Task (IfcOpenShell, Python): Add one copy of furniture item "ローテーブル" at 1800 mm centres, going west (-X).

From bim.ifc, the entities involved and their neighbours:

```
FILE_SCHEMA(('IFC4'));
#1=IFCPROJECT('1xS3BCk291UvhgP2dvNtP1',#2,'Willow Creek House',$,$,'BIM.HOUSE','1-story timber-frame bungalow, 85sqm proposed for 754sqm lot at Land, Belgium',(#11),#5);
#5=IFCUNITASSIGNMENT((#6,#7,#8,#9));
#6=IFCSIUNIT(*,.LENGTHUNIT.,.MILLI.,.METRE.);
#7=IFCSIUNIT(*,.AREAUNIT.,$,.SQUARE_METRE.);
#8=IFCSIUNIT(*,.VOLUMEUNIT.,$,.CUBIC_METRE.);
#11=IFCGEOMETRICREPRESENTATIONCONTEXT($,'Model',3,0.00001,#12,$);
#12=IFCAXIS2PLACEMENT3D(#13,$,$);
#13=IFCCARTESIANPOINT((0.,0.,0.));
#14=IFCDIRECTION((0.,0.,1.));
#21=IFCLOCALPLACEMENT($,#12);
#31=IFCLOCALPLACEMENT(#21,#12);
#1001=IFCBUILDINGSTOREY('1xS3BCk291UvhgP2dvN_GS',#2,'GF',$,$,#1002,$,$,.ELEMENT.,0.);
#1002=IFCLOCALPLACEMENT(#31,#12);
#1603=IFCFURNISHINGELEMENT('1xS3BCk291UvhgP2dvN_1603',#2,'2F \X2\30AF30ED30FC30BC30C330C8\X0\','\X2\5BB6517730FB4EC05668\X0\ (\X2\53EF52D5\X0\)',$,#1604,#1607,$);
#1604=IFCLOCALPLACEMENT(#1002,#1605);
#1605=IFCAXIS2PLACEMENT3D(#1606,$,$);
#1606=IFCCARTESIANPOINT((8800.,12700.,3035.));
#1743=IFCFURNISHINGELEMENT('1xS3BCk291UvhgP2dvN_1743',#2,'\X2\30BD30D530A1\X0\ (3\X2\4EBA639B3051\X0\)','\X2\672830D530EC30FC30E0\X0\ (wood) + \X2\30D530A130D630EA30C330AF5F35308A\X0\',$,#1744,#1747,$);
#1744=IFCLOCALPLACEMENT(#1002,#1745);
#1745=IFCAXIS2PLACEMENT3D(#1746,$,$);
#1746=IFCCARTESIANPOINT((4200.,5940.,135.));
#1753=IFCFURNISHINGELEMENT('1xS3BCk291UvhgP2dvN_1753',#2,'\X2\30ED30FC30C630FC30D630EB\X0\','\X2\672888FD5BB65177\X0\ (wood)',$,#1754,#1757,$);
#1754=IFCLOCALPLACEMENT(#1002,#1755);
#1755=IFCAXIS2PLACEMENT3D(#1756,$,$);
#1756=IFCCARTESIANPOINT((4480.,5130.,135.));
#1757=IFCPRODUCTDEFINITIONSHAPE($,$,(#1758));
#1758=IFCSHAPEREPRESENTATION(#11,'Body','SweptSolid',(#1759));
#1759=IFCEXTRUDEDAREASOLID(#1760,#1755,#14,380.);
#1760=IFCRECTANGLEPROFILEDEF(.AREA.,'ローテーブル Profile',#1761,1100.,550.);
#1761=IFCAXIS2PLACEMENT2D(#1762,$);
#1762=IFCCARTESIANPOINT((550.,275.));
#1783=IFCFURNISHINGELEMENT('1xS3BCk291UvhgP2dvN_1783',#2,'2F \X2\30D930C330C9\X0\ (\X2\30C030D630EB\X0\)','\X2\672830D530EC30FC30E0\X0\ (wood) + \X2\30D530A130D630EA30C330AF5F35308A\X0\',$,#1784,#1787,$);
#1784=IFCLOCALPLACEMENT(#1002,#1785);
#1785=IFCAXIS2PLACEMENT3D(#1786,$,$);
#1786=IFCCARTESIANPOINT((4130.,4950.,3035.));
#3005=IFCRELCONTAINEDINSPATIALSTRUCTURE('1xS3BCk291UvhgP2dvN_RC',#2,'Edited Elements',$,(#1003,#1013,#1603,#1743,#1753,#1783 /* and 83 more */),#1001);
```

```python
import numpy as np
import ifcopenshell
import ifcopenshell.api.geometry
import ifcopenshell.api.root
import ifcopenshell.util.element
import ifcopenshell.util.placement
import ifcopenshell.util.unit

model = ifcopenshell.open("bim.ifc")
unit_scale = ifcopenshell.util.unit.calculate_unit_scale(model)


def reuse_history(source, copy):
    """copy_class also copies each property set's owner history, people and application; keep the originals."""
    for rel in copy.IsDefinedBy:
        if rel.is_a("IfcRelDefinesByProperties") and (history := rel.RelatingPropertyDefinition.OwnerHistory):
            rel.RelatingPropertyDefinition.OwnerHistory = source.OwnerHistory
            ifcopenshell.util.element.remove_deep2(model, history)


source = model.by_guid("1xS3BCk291UvhgP2dvN_1753")
base = ifcopenshell.util.placement.get_local_placement(source.ObjectPlacement)
step = np.array([-1.0, 0.0, 0.0]) * 1.8 / unit_scale

for i in range(1, 2):
    copy = ifcopenshell.api.root.copy_class(model, product=source)
    copy.Representation = ifcopenshell.util.element.copy_deep(
        model, source.Representation, exclude=["IfcGeometricRepresentationContext", "IfcRepresentationMap"]
    )
    reuse_history(source, copy)
    matrix = base.copy()
    matrix[:3, 3] += i * step
    print("added at", matrix[:3, 3].round(3) + 0.0)
    ifcopenshell.api.geometry.edit_object_placement(model, product=copy, matrix=matrix, is_si=False)

model.write("bim-out.ifc")
```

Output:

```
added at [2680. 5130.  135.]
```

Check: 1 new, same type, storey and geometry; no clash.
